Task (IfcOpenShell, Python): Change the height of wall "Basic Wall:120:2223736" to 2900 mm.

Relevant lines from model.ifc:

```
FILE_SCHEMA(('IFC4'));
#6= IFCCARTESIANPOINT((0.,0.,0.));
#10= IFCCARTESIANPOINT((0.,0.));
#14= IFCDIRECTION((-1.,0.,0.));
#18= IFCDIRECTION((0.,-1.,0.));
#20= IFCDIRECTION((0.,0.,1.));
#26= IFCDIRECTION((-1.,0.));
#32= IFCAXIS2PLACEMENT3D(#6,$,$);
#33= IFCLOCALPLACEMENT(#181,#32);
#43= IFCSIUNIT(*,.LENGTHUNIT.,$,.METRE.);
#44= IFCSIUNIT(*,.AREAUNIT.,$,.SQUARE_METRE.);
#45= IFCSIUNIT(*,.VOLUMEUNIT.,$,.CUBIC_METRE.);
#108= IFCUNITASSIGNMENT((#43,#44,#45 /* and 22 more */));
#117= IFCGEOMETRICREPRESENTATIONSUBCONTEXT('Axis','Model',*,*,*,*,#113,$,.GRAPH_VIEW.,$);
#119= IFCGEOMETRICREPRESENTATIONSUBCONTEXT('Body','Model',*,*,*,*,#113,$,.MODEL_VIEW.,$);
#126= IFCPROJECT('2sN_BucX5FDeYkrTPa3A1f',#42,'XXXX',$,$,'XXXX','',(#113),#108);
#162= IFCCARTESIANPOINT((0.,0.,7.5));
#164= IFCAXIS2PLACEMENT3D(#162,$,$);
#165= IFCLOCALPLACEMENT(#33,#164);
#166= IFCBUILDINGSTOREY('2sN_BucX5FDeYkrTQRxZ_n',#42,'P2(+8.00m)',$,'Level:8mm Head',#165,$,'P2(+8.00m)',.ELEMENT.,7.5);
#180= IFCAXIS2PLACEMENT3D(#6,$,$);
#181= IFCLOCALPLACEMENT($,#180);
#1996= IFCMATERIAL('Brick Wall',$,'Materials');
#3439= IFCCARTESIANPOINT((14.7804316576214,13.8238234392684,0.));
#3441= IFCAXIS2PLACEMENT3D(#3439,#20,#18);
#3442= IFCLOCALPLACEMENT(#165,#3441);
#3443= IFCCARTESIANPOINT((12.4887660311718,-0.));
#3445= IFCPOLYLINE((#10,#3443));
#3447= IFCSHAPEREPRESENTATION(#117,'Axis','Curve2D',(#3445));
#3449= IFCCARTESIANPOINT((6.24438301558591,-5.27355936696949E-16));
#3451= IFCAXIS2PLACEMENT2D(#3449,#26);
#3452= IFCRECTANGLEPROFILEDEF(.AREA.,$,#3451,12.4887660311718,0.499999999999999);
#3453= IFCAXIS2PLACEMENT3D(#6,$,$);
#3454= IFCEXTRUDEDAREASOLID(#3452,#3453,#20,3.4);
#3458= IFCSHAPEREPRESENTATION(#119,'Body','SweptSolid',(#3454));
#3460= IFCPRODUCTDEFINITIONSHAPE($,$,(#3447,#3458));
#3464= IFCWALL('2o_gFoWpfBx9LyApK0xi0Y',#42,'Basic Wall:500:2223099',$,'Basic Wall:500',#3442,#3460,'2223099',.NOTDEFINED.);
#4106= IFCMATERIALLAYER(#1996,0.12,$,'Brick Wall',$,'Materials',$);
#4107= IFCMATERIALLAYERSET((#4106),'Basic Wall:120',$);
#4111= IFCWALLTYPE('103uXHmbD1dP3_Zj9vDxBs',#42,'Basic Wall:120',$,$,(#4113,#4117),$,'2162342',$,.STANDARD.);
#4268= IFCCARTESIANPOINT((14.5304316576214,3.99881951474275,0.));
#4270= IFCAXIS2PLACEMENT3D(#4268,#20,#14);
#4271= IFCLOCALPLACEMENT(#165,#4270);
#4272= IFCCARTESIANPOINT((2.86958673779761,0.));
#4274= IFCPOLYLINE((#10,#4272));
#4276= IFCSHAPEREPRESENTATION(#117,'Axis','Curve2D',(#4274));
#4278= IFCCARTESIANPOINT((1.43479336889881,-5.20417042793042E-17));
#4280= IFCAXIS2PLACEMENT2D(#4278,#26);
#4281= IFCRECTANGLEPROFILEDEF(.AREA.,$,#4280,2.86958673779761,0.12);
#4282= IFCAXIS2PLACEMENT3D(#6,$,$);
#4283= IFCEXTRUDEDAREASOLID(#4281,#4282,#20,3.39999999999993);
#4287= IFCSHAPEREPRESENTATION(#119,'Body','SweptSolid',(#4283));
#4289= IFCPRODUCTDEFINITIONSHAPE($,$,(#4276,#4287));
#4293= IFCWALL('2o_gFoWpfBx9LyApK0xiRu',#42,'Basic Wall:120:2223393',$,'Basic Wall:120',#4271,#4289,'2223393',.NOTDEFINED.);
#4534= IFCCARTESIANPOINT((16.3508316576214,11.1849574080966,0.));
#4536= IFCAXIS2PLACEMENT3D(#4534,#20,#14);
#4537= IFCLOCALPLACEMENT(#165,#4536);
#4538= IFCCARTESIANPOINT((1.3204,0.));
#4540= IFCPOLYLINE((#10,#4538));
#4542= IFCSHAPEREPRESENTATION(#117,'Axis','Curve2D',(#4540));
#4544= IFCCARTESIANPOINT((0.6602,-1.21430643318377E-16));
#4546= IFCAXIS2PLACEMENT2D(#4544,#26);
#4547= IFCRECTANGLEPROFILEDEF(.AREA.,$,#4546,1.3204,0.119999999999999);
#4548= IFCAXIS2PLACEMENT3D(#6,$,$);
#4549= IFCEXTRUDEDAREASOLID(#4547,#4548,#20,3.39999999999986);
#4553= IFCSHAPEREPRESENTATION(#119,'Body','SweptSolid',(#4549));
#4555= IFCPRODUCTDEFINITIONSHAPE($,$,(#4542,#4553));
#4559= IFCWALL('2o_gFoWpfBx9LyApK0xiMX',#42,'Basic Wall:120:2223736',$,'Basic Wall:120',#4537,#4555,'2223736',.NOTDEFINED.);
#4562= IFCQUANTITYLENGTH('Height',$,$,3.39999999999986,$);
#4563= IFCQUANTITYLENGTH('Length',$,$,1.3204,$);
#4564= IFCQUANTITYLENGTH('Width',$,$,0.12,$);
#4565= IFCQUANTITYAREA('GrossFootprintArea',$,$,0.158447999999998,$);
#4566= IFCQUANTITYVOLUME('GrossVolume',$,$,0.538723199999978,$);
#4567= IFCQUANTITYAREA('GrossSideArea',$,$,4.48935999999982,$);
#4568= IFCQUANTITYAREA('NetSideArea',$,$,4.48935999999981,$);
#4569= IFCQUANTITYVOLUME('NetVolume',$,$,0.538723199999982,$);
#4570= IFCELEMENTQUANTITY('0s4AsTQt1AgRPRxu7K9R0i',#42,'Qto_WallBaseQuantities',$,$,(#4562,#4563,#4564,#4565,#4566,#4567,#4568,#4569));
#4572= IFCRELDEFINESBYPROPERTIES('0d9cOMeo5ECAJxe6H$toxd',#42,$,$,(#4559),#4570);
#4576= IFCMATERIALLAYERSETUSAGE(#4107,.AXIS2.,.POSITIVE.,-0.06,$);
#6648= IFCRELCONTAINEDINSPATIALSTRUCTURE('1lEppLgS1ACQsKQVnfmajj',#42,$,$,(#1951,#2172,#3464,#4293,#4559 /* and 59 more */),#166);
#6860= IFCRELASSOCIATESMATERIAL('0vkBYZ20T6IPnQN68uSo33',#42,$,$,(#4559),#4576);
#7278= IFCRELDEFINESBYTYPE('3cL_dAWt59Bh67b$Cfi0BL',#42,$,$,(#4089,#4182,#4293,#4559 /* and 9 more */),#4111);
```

```python
import ifcopenshell
import ifcopenshell.api.pset
import ifcopenshell.geom
import ifcopenshell.util.element
import ifcopenshell.util.representation
import ifcopenshell.util.shape
import ifcopenshell.util.unit

model = ifcopenshell.open("model.ifc")
unit_scale = ifcopenshell.util.unit.calculate_unit_scale(model)
area_scale = ifcopenshell.util.unit.calculate_unit_scale(model, "AREAUNIT")
volume_scale = ifcopenshell.util.unit.calculate_unit_scale(model, "VOLUMEUNIT")
settings = ifcopenshell.geom.settings()


def volume(element):
    """Net volume in cubic metres, openings subtracted."""
    shape = ifcopenshell.geom.create_shape(settings, element)
    return ifcopenshell.util.shape.get_volume(shape.geometry)


wall = model.by_guid("2o_gFoWpfBx9LyApK0xiMX")
before = volume(wall)

body = ifcopenshell.util.representation.get_representation(wall, "Model", "Body")
solid = body.Items[0]
old_height = solid.Depth
solid.Depth = 2.9 / unit_scale
after = volume(wall)
thickness = 0.12  # wall thickness in metres

# Update the stored height, areas and volumes.
qto = model.by_id(ifcopenshell.util.element.get_pset(wall, "Qto_WallBaseQuantities", should_inherit=False)["id"])
ifcopenshell.api.pset.edit_qto(model, qto=qto, properties={
    "Height": solid.Depth,
    "GrossVolume": ifcopenshell.util.element.get_pset(wall, "Qto_WallBaseQuantities", "GrossVolume") * solid.Depth / old_height,
    "GrossSideArea": ifcopenshell.util.element.get_pset(wall, "Qto_WallBaseQuantities", "GrossSideArea") * solid.Depth / old_height,
    "NetSideArea": after / thickness / area_scale,
    "NetVolume": after / volume_scale,
})

print(f"height {old_height:g} -> {solid.Depth:g}, volume {before:.3f} -> {after:.3f} m3")

model.write("model_edited.ifc")
```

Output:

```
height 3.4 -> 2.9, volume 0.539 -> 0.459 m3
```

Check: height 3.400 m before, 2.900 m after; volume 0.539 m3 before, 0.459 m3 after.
